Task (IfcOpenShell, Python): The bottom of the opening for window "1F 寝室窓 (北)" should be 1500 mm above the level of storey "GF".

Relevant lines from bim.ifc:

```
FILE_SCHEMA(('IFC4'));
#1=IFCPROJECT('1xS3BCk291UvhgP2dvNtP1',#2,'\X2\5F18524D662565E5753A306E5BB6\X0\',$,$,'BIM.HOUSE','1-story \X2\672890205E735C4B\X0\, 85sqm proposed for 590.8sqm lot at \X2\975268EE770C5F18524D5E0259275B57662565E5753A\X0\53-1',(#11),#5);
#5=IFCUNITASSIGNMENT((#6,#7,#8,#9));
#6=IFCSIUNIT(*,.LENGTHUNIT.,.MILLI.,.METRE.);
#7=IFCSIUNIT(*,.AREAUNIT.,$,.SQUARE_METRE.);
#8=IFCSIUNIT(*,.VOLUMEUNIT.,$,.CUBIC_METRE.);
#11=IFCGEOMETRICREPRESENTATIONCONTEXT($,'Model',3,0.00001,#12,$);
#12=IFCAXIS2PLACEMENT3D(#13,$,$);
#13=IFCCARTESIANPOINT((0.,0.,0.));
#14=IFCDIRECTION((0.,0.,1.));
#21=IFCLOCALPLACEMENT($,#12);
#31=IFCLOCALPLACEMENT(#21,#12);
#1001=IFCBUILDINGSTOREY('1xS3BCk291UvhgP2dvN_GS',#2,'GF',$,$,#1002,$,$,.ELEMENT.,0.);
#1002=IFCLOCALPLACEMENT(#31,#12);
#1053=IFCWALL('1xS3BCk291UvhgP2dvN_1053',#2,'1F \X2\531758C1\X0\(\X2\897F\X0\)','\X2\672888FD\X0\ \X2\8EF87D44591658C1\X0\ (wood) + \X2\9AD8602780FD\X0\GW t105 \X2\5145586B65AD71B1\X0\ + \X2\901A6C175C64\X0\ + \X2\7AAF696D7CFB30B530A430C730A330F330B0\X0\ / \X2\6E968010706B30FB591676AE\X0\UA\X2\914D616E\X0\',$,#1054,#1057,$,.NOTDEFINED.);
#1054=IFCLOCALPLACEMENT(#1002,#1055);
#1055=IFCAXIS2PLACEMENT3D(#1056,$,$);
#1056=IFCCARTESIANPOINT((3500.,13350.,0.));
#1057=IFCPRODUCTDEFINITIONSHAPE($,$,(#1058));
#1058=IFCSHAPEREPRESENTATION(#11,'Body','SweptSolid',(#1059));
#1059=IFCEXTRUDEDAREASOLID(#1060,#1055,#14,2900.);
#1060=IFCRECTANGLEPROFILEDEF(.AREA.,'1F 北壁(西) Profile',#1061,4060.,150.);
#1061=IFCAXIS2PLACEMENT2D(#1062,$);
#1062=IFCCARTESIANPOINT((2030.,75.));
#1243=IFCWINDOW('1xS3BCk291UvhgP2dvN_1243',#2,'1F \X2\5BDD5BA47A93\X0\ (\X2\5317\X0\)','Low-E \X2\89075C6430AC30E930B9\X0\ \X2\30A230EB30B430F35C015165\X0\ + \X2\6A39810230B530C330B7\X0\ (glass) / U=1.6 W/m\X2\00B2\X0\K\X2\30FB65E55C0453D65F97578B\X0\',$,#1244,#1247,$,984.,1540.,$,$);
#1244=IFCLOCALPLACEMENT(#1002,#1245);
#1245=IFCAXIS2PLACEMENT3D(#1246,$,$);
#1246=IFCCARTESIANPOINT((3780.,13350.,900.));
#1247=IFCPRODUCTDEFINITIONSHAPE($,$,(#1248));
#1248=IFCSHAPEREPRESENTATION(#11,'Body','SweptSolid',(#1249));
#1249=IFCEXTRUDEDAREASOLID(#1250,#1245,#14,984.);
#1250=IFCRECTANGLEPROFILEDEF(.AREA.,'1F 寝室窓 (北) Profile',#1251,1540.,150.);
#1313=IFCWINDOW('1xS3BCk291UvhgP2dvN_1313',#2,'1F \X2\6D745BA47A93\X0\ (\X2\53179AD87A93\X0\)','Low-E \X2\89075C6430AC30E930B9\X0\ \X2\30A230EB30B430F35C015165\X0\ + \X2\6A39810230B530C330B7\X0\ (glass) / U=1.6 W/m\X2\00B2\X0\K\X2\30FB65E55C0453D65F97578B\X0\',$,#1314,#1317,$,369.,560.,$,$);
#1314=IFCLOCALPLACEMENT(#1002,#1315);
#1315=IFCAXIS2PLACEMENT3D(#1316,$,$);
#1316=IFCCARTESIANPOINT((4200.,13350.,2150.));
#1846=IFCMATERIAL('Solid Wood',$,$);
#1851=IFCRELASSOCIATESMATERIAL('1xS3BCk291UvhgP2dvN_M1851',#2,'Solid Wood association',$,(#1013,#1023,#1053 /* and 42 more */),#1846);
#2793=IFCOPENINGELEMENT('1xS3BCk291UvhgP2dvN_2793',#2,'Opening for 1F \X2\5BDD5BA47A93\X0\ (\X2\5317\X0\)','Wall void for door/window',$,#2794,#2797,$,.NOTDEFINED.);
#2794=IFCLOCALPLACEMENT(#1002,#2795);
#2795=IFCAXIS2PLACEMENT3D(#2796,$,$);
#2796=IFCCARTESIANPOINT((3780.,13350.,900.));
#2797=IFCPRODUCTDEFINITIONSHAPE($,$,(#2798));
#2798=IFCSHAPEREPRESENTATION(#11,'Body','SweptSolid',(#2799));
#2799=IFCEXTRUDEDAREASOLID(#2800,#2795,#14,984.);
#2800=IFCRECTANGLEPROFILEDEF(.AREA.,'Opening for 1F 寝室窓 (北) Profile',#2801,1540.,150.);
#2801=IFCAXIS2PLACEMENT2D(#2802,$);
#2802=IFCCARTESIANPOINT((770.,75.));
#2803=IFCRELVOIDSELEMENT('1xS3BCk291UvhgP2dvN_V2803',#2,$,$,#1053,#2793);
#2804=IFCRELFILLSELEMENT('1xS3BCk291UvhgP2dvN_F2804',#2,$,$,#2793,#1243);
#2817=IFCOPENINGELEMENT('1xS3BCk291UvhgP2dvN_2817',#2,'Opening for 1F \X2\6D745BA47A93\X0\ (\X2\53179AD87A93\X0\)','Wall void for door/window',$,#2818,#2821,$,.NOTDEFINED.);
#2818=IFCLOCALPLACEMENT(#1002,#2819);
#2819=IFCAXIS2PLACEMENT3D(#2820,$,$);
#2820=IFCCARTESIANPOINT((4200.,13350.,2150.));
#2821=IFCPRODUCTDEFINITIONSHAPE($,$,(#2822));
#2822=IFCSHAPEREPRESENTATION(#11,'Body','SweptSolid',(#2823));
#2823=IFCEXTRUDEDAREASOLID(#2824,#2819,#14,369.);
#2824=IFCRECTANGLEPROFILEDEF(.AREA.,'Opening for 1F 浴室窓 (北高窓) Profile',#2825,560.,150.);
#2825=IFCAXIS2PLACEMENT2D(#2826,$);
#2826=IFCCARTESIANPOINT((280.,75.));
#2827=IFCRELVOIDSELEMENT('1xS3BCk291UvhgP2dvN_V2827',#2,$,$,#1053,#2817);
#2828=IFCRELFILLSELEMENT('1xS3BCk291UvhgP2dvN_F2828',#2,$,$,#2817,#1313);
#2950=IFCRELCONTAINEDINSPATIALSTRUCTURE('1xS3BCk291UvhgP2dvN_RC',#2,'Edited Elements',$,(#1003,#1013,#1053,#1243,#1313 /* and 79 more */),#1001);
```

```python
import numpy as np
import ifcopenshell
import ifcopenshell.api.geometry
import ifcopenshell.geom
import ifcopenshell.util.element
import ifcopenshell.util.placement
import ifcopenshell.util.shape
import ifcopenshell.util.unit

model = ifcopenshell.open("bim.ifc")
unit_scale = ifcopenshell.util.unit.calculate_unit_scale(model)

window = model.by_guid("1xS3BCk291UvhgP2dvN_1243")
opening = window.FillsVoids[0].RelatingOpeningElement
storey = ifcopenshell.util.element.get_container(window, ifc_class="IfcBuildingStorey")
level = ifcopenshell.util.placement.get_local_placement(storey.ObjectPlacement)[2, 3]

# The opening's origin need not be at the sill, so measure its lowest point.
shape = ifcopenshell.geom.create_shape(ifcopenshell.geom.settings(), opening)
bottom = ifcopenshell.util.shape.get_shape_bottom_elevation(shape, shape.geometry) / unit_scale
dz = level + 1.5 / unit_scale - bottom

shift = np.array([0.0, 0.0, dz])
# The window is not placed relative to its opening, so move both.
for product in (opening, window):
    matrix = ifcopenshell.util.placement.get_local_placement(product.ObjectPlacement)
    matrix[:3, 3] += shift
    ifcopenshell.api.geometry.edit_object_placement(model, product=product, matrix=matrix, is_si=False)

print(f"moved by {dz * unit_scale:+.3f} m")

model.write("bim_edited.ifc")
```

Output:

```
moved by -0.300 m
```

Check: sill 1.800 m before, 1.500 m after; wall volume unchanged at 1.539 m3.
